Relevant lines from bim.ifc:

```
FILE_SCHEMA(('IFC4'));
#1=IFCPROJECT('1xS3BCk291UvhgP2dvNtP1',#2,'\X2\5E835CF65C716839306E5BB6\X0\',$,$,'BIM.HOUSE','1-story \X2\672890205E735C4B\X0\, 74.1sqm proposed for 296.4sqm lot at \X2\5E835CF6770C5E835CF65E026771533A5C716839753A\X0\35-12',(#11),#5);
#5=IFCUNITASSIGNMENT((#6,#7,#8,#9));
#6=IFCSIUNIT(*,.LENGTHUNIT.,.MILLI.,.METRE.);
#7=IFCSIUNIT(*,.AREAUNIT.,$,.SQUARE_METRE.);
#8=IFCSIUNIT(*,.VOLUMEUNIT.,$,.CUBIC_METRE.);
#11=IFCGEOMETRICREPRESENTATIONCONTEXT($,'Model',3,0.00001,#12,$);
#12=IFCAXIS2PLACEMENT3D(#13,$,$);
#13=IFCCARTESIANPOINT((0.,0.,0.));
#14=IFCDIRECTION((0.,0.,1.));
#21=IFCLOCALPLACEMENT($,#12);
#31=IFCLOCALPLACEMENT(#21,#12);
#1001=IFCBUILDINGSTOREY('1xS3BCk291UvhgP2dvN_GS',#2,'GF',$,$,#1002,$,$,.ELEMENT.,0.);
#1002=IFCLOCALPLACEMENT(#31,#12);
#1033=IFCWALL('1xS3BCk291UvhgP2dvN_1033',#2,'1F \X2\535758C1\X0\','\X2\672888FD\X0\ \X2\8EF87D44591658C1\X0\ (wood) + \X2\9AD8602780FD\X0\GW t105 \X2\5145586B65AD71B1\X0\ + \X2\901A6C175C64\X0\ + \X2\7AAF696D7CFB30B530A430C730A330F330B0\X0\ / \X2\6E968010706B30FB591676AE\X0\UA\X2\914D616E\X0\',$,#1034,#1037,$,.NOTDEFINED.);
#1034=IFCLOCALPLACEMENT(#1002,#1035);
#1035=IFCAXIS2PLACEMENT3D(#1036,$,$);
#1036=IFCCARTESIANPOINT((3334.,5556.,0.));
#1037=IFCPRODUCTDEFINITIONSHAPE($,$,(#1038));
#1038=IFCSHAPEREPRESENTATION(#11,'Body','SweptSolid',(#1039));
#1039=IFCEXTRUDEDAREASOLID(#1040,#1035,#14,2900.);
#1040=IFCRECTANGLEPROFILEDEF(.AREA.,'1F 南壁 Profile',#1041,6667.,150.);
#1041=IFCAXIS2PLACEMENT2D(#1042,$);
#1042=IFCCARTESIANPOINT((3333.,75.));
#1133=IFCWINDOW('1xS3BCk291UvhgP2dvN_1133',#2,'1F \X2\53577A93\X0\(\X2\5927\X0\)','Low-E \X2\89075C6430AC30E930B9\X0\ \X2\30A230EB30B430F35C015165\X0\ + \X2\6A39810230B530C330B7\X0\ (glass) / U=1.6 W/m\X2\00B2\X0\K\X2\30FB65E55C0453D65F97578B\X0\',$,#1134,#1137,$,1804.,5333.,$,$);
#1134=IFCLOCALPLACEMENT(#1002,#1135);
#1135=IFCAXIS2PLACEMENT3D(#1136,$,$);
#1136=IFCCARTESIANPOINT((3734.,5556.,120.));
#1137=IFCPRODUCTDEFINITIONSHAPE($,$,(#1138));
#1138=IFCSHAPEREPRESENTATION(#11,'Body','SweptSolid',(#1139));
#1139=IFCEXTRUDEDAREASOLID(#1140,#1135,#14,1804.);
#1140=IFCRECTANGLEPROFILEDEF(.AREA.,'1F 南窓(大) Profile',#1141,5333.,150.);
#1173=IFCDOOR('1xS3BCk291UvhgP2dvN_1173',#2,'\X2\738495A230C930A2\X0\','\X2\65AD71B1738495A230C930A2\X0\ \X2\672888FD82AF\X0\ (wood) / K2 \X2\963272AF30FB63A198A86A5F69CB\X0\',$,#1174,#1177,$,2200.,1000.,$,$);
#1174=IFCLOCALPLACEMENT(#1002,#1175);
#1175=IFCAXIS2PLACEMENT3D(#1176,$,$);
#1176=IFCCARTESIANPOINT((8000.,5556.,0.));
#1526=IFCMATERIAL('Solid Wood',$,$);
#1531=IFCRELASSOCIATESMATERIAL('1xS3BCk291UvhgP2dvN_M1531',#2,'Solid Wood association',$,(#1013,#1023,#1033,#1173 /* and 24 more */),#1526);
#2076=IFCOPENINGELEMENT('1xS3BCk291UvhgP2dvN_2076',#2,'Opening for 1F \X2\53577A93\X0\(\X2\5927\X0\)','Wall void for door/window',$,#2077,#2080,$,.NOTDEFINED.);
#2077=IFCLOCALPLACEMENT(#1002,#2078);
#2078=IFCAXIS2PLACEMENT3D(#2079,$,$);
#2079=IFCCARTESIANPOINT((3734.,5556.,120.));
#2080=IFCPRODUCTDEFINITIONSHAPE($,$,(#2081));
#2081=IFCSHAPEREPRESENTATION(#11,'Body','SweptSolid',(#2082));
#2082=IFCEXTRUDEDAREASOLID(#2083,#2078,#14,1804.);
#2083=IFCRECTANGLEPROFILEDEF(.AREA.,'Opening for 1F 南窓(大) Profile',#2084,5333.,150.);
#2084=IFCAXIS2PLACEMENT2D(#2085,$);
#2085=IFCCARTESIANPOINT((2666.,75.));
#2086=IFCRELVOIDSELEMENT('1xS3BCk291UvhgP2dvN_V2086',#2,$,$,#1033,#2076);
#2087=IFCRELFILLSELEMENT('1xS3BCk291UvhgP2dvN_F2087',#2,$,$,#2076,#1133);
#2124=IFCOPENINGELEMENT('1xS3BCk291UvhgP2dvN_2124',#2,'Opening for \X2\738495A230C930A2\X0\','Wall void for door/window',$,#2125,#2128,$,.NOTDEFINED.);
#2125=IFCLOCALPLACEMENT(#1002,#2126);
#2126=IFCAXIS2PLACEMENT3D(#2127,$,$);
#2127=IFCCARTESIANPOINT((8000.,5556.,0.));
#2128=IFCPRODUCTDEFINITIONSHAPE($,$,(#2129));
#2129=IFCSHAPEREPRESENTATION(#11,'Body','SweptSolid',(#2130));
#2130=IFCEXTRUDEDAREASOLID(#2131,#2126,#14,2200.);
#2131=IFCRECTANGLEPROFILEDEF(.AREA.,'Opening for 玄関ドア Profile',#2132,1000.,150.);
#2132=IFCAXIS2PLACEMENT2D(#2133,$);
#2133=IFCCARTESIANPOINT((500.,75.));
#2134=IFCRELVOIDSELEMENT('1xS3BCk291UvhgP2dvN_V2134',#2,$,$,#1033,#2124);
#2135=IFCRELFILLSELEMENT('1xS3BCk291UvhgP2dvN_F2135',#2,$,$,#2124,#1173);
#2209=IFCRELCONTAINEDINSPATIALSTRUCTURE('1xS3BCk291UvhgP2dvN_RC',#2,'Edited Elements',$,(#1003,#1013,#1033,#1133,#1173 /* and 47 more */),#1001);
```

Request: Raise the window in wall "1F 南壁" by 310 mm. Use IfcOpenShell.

```python
import numpy as np
import ifcopenshell
import ifcopenshell.api.geometry
import ifcopenshell.util.placement
import ifcopenshell.util.unit

model = ifcopenshell.open("bim.ifc")
unit_scale = ifcopenshell.util.unit.calculate_unit_scale(model)

window = model.by_id(1133)
opening = window.FillsVoids[0].RelatingOpeningElement
dz = 0.31 / unit_scale

shift = np.array([0.0, 0.0, dz])
# The window is not placed relative to its opening, so move both.
for product in (opening, window):
    matrix = ifcopenshell.util.placement.get_local_placement(product.ObjectPlacement)
    matrix[:3, 3] += shift
    ifcopenshell.api.geometry.edit_object_placement(model, product=product, matrix=matrix, is_si=False)

print(f"moved by {dz * unit_scale:+.3f} m")

model.write("bim_updated.ifc")
```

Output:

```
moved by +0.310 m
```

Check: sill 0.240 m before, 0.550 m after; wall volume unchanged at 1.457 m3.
